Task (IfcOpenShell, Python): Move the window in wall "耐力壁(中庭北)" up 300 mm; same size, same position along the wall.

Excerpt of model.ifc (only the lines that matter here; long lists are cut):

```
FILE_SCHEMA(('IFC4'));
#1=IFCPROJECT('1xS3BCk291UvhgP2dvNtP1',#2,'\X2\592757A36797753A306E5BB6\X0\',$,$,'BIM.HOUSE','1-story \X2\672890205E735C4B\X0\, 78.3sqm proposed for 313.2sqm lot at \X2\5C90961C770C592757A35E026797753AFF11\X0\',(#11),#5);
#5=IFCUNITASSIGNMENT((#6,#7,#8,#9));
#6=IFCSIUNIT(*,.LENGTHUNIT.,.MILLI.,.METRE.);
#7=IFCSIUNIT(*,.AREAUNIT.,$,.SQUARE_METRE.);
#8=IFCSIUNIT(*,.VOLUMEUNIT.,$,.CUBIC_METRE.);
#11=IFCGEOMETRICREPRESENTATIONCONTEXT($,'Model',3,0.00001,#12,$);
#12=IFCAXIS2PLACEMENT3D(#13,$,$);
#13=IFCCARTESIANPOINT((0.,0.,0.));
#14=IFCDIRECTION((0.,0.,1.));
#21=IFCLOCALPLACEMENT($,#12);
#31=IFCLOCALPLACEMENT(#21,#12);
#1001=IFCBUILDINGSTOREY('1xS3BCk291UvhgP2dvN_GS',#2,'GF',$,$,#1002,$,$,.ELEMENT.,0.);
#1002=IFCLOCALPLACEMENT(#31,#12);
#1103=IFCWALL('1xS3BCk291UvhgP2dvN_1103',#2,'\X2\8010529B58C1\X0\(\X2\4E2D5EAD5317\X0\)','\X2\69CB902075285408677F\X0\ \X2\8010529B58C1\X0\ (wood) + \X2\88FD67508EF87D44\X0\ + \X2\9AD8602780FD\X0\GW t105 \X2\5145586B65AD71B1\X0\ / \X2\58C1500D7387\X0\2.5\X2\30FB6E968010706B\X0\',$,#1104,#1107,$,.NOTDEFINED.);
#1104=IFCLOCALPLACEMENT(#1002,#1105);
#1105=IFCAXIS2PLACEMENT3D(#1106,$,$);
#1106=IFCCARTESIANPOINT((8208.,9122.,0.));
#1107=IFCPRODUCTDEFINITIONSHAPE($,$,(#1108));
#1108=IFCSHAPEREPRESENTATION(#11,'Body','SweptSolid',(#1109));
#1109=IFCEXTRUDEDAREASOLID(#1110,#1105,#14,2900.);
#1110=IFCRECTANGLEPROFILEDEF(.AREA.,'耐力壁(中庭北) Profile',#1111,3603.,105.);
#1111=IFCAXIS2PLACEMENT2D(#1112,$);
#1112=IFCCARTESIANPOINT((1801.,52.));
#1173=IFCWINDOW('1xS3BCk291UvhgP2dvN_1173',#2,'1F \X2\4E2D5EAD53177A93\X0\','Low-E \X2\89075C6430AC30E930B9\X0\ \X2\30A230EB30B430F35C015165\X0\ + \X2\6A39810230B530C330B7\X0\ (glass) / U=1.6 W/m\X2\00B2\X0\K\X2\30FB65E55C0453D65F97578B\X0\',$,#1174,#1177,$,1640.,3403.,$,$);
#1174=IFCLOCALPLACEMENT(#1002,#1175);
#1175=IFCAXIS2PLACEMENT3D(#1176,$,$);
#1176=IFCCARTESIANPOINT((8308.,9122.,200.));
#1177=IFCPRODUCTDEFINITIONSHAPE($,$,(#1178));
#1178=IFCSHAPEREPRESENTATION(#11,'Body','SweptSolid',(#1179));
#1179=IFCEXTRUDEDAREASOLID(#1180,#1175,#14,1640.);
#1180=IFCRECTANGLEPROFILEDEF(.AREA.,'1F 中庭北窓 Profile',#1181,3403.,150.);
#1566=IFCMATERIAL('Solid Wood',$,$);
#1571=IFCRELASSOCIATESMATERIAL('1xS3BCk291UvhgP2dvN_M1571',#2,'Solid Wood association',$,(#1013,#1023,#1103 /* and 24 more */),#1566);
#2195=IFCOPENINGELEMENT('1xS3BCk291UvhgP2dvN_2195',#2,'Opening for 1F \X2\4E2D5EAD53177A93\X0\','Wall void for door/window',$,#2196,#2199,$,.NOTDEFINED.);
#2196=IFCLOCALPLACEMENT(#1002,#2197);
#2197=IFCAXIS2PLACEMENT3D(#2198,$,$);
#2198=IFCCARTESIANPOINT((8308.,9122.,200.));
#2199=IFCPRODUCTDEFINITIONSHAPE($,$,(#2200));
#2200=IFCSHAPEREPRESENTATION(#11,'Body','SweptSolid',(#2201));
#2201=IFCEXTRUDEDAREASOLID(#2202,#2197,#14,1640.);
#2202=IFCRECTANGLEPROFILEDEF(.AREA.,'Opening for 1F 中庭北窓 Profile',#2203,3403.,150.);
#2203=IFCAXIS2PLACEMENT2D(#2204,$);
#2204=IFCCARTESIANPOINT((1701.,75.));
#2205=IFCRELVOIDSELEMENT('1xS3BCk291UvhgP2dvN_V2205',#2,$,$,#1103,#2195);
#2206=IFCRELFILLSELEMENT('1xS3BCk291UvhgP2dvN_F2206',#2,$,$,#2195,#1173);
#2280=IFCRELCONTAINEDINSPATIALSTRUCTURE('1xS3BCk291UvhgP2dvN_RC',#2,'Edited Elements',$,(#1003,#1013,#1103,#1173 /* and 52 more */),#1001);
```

```python
import numpy as np
import ifcopenshell
import ifcopenshell.api.geometry
import ifcopenshell.util.placement
import ifcopenshell.util.unit

model = ifcopenshell.open("model.ifc")
unit_scale = ifcopenshell.util.unit.calculate_unit_scale(model)

window = model.by_guid("1xS3BCk291UvhgP2dvN_1173")
opening = window.FillsVoids[0].RelatingOpeningElement
dz = 0.3 / unit_scale

shift = np.array([0.0, 0.0, dz])
# The window is not placed relative to its opening, so move both.
for product in (opening, window):
    matrix = ifcopenshell.util.placement.get_local_placement(product.ObjectPlacement)
    matrix[:3, 3] += shift
    ifcopenshell.api.geometry.edit_object_placement(model, product=product, matrix=matrix, is_si=False)

print(f"moved by {dz * unit_scale:+.3f} m")

model.write("model_v2.ifc")
```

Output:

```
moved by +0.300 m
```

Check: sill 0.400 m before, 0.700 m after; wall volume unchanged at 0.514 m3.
